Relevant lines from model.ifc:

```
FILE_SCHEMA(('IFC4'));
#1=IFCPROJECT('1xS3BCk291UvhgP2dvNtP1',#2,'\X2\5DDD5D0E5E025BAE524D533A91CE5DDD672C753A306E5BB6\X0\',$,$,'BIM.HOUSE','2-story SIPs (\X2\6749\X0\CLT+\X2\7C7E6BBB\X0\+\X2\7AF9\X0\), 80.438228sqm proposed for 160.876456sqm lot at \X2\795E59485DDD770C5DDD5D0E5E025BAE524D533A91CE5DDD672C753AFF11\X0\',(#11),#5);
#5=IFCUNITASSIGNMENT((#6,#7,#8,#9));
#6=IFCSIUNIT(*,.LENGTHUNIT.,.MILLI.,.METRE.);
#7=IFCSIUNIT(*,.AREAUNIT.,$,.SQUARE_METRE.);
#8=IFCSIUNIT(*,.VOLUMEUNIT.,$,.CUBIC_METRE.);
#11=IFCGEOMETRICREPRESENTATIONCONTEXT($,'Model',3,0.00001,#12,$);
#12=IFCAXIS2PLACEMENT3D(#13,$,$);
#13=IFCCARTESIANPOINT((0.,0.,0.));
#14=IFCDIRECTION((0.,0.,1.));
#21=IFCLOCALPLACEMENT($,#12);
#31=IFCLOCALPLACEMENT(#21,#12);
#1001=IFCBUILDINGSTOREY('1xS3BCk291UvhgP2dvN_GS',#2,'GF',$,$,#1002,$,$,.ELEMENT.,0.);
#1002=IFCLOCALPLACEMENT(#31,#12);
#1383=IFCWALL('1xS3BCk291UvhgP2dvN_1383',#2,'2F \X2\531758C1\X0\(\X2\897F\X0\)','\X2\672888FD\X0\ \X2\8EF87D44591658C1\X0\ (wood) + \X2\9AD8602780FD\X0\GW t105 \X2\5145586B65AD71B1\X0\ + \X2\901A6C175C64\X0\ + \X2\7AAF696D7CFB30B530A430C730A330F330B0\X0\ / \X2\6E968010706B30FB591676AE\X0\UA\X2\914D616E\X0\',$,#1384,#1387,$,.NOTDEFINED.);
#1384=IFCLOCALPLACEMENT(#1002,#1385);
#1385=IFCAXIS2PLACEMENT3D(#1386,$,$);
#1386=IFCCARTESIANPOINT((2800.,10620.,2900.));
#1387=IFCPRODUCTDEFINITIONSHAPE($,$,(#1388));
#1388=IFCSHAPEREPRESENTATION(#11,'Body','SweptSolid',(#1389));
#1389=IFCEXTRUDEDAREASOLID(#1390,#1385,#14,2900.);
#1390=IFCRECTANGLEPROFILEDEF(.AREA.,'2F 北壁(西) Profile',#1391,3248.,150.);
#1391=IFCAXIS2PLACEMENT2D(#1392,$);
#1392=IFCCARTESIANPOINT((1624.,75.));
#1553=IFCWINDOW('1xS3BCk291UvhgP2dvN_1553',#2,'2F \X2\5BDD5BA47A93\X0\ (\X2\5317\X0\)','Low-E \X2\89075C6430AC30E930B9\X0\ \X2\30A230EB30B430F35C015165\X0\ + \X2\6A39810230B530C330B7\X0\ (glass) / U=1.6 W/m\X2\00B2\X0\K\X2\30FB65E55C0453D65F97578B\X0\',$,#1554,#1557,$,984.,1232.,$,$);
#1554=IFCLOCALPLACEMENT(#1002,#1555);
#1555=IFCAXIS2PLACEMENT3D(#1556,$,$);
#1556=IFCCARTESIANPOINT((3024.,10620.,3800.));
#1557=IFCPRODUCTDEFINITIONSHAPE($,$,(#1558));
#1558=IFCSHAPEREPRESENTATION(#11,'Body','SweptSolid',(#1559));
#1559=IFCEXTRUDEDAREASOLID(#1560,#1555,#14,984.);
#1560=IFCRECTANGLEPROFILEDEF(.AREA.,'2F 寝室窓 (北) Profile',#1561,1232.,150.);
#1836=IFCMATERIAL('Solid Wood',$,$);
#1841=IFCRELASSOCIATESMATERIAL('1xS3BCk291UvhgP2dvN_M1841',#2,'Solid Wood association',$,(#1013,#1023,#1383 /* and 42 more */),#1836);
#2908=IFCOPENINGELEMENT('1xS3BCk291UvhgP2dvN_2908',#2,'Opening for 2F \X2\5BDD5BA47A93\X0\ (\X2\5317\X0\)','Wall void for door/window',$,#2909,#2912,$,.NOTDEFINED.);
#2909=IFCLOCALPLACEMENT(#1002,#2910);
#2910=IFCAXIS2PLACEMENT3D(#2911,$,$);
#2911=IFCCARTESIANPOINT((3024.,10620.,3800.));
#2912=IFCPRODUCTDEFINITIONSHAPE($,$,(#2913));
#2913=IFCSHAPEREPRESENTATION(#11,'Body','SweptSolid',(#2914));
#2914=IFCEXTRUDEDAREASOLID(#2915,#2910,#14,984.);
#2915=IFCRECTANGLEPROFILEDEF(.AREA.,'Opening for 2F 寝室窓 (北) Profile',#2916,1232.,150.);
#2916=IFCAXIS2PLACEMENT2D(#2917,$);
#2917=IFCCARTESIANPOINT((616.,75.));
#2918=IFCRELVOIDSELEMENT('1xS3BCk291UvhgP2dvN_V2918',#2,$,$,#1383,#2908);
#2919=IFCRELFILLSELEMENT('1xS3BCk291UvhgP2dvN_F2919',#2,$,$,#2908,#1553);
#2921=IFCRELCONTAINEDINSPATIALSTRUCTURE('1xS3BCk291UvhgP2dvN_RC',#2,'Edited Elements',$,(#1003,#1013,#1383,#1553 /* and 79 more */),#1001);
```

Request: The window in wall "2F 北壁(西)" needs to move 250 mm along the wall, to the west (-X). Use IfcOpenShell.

```python
import ifcopenshell
import ifcopenshell.api.geometry
import ifcopenshell.util.placement

model = ifcopenshell.open("model.ifc")

window = model.by_guid("1xS3BCk291UvhgP2dvN_1553")
opening = window.FillsVoids[0].RelatingOpeningElement
wall = opening.VoidsElements[0].RelatingBuildingElement

wall_matrix = ifcopenshell.util.placement.get_local_placement(wall.ObjectPlacement)
shift = wall_matrix[:3, 0] * -250.0
before = ifcopenshell.util.placement.get_local_placement(window.ObjectPlacement)[:3, 3].copy()

# The window is not placed relative to its opening, so move both.
for product in (opening, window):
    matrix = ifcopenshell.util.placement.get_local_placement(product.ObjectPlacement)
    matrix[:3, 3] += shift
    ifcopenshell.api.geometry.edit_object_placement(model, product=product, matrix=matrix, is_si=False)

after = ifcopenshell.util.placement.get_local_placement(window.ObjectPlacement)[:3, 3]
print("window moved by", (after - before).round(3) + 0.0)

model.write("model-out.ifc")
```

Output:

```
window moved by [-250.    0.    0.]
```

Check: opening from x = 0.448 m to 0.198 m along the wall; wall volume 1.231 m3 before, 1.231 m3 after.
